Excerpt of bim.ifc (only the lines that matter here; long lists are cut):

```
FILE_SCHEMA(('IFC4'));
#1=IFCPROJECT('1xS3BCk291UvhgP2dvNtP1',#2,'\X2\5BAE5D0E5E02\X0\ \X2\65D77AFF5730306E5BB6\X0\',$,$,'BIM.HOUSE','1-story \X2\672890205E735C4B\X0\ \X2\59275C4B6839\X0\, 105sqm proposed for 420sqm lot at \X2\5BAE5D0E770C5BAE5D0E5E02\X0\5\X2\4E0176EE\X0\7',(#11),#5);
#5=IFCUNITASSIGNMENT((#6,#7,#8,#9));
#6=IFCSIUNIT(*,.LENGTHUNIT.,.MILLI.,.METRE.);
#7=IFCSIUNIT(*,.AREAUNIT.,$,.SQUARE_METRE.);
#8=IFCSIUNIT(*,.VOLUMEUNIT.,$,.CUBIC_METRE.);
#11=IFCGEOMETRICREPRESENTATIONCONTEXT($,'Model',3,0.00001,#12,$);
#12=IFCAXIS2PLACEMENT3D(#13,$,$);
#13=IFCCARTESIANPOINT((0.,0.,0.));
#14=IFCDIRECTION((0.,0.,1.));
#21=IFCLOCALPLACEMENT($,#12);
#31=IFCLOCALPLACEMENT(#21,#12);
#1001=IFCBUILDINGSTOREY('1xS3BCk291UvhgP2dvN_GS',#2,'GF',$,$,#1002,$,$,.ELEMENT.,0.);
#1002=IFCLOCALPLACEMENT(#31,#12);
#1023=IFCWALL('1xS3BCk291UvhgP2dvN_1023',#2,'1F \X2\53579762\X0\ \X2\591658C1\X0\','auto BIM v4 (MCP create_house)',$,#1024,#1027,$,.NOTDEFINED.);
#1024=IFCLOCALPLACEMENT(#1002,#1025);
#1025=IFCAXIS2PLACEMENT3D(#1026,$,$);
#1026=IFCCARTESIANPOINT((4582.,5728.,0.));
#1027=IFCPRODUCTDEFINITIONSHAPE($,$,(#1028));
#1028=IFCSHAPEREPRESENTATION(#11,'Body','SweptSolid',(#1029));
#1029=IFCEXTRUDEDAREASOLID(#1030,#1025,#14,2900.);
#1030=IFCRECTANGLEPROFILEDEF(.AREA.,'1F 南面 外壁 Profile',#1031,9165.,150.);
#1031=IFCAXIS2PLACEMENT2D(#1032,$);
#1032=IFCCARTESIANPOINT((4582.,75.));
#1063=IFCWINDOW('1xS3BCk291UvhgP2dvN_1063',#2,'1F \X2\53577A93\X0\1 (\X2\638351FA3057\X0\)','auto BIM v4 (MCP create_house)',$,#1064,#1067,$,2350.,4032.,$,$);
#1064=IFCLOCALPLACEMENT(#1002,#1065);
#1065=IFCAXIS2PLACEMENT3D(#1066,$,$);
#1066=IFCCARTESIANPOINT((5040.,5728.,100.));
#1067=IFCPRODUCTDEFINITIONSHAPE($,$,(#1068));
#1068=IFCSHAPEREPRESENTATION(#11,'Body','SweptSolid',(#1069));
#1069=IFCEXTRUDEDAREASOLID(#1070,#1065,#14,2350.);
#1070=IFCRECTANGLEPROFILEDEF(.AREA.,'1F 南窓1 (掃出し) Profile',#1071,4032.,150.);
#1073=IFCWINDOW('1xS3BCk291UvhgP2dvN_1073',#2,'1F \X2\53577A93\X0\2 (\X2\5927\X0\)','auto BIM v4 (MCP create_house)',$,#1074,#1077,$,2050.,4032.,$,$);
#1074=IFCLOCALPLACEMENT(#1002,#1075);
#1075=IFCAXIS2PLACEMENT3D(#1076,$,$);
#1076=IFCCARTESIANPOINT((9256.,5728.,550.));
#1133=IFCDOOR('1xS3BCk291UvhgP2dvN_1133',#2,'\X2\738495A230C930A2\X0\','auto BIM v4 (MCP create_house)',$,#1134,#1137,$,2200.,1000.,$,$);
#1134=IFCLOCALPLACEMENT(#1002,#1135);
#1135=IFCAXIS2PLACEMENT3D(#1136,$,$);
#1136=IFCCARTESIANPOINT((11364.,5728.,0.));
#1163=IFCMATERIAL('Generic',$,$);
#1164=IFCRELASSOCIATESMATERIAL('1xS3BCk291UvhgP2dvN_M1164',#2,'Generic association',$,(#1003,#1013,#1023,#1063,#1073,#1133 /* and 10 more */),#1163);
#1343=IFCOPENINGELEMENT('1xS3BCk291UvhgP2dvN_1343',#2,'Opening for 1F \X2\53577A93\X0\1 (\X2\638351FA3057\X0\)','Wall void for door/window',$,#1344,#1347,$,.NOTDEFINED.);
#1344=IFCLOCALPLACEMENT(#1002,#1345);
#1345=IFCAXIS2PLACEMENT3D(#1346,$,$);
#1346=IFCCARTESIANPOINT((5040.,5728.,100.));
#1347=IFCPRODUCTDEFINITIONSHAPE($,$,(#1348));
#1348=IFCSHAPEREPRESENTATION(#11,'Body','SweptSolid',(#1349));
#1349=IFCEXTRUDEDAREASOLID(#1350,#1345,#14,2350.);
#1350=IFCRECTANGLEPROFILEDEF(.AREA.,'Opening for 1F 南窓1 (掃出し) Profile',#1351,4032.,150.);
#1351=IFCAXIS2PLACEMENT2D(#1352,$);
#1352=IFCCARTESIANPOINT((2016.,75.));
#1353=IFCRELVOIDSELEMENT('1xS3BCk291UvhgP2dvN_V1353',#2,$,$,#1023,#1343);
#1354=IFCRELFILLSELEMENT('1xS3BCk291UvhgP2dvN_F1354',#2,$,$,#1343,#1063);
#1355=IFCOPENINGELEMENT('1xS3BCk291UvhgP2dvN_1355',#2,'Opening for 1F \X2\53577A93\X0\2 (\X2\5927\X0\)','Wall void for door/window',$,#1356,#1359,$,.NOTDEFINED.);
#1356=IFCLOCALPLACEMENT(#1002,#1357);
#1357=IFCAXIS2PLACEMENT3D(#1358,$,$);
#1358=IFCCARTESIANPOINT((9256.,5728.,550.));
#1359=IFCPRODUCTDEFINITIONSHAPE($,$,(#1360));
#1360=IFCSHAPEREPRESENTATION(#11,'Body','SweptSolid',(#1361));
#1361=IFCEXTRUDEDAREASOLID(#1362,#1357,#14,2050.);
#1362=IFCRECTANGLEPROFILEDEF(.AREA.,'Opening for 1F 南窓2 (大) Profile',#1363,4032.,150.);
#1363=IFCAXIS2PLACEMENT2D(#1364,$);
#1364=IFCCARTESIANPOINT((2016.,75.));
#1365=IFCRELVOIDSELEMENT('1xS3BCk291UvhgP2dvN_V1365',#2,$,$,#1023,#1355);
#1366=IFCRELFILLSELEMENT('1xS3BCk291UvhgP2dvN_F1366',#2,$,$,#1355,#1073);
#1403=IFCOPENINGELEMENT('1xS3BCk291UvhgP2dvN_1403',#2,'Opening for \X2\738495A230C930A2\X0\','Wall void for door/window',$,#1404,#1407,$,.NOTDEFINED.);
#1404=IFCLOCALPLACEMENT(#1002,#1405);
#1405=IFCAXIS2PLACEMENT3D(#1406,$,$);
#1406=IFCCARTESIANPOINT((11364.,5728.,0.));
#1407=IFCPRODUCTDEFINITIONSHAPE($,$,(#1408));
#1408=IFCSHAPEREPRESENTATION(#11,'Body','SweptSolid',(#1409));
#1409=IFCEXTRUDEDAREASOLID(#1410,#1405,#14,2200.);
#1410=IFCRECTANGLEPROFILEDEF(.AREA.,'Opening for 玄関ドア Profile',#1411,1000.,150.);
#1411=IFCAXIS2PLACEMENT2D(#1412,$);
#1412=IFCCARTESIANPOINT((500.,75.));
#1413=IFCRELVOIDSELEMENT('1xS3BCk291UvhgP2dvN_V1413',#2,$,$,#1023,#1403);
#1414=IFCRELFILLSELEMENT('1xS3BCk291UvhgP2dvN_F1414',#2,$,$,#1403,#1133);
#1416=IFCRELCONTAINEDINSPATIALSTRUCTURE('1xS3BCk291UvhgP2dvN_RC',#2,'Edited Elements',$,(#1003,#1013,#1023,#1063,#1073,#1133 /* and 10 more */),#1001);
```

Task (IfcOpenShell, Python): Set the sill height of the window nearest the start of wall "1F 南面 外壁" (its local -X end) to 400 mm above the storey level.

```python
import numpy as np
import ifcopenshell
import ifcopenshell.api.geometry
import ifcopenshell.geom
import ifcopenshell.util.element
import ifcopenshell.util.placement
import ifcopenshell.util.shape
import ifcopenshell.util.unit

model = ifcopenshell.open("bim.ifc")
unit_scale = ifcopenshell.util.unit.calculate_unit_scale(model)

window = model.by_guid("1xS3BCk291UvhgP2dvN_1063")
opening = window.FillsVoids[0].RelatingOpeningElement
storey = ifcopenshell.util.element.get_container(window, ifc_class="IfcBuildingStorey")
level = ifcopenshell.util.placement.get_local_placement(storey.ObjectPlacement)[2, 3]

# The opening's origin need not be at the sill, so measure its lowest point.
shape = ifcopenshell.geom.create_shape(ifcopenshell.geom.settings(), opening)
bottom = ifcopenshell.util.shape.get_shape_bottom_elevation(shape, shape.geometry) / unit_scale
dz = level + 400.0 - bottom

shift = np.array([0.0, 0.0, dz])
# The window is not placed relative to its opening, so move both.
for product in (opening, window):
    matrix = ifcopenshell.util.placement.get_local_placement(product.ObjectPlacement)
    matrix[:3, 3] += shift
    ifcopenshell.api.geometry.edit_object_placement(model, product=product, matrix=matrix, is_si=False)

print(f"moved by {dz * unit_scale:+.3f} m")

model.write("bim_edited.ifc")
```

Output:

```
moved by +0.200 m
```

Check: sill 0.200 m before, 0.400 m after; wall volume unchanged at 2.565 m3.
